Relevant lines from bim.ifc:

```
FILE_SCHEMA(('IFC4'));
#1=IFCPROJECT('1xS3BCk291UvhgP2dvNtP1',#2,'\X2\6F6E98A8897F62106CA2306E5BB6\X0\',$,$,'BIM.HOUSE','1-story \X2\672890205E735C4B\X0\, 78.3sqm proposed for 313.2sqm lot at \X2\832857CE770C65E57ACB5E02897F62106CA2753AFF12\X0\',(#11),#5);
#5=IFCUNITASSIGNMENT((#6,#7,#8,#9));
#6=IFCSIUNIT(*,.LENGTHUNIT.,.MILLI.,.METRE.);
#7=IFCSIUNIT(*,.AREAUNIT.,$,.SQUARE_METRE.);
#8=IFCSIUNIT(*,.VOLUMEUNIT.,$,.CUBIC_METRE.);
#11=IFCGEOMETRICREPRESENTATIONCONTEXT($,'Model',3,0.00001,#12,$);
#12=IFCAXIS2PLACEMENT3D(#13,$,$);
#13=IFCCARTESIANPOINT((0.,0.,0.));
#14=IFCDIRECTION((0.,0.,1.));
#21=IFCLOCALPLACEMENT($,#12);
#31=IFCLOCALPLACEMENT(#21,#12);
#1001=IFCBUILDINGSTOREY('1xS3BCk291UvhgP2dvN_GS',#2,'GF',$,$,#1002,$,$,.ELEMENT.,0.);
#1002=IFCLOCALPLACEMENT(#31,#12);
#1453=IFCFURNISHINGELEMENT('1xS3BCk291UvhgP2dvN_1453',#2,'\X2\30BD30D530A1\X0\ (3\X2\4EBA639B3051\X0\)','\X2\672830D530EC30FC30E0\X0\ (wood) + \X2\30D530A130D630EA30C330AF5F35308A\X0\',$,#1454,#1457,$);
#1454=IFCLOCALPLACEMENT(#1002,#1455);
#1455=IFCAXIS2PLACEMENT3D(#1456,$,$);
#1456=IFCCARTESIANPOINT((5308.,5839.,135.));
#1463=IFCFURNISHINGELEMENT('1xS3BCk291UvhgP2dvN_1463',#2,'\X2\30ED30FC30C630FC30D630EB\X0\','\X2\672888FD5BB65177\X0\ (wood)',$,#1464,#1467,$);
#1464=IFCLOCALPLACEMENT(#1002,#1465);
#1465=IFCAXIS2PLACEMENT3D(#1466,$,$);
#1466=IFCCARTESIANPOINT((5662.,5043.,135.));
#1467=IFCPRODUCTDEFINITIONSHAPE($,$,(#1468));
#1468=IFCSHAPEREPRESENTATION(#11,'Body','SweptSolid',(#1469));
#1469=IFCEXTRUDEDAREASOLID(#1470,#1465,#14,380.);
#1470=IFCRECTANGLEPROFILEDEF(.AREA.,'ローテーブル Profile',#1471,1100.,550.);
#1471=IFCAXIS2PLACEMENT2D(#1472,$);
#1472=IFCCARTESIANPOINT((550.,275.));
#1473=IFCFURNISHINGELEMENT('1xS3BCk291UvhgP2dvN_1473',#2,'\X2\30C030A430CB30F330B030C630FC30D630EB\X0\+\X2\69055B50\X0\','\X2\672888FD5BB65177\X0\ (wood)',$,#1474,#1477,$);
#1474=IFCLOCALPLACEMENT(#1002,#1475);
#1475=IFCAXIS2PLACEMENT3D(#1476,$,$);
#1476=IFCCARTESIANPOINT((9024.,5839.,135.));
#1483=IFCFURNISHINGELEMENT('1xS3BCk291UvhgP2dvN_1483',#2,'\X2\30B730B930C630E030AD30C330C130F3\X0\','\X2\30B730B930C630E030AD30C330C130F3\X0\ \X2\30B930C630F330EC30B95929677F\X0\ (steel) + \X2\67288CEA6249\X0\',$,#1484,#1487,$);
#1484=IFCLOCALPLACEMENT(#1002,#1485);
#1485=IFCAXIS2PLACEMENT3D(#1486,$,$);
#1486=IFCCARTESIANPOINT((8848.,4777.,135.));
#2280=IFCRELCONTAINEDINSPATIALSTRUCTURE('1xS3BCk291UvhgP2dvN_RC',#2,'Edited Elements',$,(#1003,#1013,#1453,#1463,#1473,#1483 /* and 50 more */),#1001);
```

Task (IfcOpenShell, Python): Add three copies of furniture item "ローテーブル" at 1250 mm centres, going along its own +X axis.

```python
import ifcopenshell
import ifcopenshell.api.geometry
import ifcopenshell.api.root
import ifcopenshell.util.element
import ifcopenshell.util.placement
import ifcopenshell.util.unit

model = ifcopenshell.open("bim.ifc")
unit_scale = ifcopenshell.util.unit.calculate_unit_scale(model)


def reuse_history(source, copy):
    """copy_class also copies each property set's owner history, people and application; keep the originals."""
    for rel in copy.IsDefinedBy:
        if rel.is_a("IfcRelDefinesByProperties") and (history := rel.RelatingPropertyDefinition.OwnerHistory):
            rel.RelatingPropertyDefinition.OwnerHistory = source.OwnerHistory
            ifcopenshell.util.element.remove_deep2(model, history)


source = model.by_guid("1xS3BCk291UvhgP2dvN_1463")
base = ifcopenshell.util.placement.get_local_placement(source.ObjectPlacement)
step = base[:3, 0] * 1.25 / unit_scale

for i in range(1, 4):
    copy = ifcopenshell.api.root.copy_class(model, product=source)
    copy.Representation = ifcopenshell.util.element.copy_deep(
        model, source.Representation, exclude=["IfcGeometricRepresentationContext", "IfcRepresentationMap"]
    )
    reuse_history(source, copy)
    matrix = base.copy()
    matrix[:3, 3] += i * step
    print("added at", matrix[:3, 3].round(3) + 0.0)
    ifcopenshell.api.geometry.edit_object_placement(model, product=copy, matrix=matrix, is_si=False)

model.write("bim_updated.ifc")
```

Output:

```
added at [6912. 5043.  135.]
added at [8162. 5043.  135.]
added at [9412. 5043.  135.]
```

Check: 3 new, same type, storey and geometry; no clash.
